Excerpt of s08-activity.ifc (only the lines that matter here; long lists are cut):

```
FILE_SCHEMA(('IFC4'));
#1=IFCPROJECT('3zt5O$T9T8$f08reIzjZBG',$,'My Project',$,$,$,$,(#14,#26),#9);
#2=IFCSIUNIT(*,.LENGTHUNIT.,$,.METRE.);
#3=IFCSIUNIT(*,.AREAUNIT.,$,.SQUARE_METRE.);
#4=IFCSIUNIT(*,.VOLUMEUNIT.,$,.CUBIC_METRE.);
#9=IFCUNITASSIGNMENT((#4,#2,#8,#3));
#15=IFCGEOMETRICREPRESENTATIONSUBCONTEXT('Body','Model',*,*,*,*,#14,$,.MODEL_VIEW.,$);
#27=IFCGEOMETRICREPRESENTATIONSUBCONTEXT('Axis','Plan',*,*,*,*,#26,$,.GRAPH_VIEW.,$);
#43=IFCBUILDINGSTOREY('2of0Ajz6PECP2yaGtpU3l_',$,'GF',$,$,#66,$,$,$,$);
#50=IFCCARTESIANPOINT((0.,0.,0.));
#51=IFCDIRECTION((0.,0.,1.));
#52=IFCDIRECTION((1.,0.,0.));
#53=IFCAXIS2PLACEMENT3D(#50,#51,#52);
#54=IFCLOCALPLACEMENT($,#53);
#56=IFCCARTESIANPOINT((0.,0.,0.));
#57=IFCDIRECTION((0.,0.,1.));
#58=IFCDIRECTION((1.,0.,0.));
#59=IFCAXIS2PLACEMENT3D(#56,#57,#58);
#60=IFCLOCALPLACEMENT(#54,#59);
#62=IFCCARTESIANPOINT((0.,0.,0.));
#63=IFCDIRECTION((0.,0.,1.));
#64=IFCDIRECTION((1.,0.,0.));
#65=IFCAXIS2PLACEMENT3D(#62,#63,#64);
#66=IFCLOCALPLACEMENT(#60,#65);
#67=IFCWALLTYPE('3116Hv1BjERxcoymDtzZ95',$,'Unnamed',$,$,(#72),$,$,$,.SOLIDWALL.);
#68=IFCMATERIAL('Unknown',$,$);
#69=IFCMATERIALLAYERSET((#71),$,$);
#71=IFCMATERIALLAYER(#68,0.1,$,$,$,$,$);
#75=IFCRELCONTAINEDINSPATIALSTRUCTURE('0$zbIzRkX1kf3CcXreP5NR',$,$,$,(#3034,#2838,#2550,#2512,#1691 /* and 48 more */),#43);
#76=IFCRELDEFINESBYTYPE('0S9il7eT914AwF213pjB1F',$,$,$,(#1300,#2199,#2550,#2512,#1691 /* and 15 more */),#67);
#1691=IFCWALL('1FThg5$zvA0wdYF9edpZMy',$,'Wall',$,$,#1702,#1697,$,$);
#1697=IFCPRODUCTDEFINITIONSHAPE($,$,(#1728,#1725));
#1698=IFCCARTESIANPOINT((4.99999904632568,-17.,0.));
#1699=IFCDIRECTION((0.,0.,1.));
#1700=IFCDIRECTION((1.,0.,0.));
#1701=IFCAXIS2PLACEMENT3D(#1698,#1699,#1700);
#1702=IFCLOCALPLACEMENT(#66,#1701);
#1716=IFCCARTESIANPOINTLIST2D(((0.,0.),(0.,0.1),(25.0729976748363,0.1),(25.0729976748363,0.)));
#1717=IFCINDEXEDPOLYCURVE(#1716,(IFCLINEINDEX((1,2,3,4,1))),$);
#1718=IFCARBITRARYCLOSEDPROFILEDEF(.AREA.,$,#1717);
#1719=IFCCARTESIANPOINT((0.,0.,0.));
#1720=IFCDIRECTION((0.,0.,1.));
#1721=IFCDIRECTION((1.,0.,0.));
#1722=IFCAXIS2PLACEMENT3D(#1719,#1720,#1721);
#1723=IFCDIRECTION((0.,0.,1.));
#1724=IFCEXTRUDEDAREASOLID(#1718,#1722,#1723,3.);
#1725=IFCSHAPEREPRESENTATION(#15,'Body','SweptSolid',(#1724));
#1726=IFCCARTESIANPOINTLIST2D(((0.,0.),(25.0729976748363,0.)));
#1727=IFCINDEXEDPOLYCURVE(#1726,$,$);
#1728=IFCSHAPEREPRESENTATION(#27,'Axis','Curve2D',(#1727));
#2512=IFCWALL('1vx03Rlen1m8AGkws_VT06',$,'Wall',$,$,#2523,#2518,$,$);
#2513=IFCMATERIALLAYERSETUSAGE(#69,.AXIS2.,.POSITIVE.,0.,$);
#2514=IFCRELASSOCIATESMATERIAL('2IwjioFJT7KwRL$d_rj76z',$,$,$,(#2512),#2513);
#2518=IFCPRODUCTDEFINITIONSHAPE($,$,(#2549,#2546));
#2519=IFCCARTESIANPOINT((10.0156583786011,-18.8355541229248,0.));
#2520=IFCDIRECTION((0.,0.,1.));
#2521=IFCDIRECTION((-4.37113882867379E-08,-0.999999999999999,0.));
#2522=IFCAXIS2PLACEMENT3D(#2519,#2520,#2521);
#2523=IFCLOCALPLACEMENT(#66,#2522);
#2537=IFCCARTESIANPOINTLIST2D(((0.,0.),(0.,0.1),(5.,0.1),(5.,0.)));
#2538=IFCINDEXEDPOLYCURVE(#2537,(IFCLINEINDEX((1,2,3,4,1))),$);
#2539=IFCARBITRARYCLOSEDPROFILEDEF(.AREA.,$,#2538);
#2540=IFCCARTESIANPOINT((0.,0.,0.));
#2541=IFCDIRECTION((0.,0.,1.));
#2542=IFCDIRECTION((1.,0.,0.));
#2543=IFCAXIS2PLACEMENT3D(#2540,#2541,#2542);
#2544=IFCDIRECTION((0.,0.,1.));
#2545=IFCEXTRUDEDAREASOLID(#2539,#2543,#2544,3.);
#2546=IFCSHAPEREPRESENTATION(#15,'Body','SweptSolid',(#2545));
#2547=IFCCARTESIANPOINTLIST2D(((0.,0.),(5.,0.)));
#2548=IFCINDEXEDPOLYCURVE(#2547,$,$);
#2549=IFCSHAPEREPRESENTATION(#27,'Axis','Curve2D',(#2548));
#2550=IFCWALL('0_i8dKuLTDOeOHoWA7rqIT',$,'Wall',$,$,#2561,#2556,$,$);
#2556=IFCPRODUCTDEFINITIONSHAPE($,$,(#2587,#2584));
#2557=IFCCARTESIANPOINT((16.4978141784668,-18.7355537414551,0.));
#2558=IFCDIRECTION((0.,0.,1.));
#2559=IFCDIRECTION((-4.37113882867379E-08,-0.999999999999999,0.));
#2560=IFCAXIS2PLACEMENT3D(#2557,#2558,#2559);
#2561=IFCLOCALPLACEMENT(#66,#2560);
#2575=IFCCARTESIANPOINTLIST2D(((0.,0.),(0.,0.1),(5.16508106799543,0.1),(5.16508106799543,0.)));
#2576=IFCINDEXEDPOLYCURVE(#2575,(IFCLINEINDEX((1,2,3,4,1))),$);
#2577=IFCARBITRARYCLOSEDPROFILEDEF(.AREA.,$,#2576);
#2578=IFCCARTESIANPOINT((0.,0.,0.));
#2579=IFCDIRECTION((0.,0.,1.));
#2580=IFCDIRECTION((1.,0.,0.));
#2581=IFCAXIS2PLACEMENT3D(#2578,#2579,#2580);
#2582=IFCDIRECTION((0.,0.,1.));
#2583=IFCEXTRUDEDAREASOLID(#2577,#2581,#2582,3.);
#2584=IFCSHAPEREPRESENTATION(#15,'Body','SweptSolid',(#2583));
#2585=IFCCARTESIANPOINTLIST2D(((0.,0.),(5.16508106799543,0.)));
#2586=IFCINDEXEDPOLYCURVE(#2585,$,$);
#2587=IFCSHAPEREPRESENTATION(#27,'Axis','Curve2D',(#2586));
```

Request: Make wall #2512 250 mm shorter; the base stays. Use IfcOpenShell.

```python
import ifcopenshell
import ifcopenshell.geom
import ifcopenshell.util.representation
import ifcopenshell.util.shape

model = ifcopenshell.open("s08-activity.ifc")
settings = ifcopenshell.geom.settings()


def volume(element):
    """Net volume in cubic metres, openings subtracted."""
    shape = ifcopenshell.geom.create_shape(settings, element)
    return ifcopenshell.util.shape.get_volume(shape.geometry)


wall = model.by_id(2512)
before = volume(wall)

body = ifcopenshell.util.representation.get_representation(wall, "Model", "Body")
solid = body.Items[0]
old_height = solid.Depth
solid.Depth -= 0.25
after = volume(wall)

print(f"height {old_height:g} -> {solid.Depth:g}, volume {before:.3f} -> {after:.3f} m3")

model.write("s08-activity_v2.ifc")
```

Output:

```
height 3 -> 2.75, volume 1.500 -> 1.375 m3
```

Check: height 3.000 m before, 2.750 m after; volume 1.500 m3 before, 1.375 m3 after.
